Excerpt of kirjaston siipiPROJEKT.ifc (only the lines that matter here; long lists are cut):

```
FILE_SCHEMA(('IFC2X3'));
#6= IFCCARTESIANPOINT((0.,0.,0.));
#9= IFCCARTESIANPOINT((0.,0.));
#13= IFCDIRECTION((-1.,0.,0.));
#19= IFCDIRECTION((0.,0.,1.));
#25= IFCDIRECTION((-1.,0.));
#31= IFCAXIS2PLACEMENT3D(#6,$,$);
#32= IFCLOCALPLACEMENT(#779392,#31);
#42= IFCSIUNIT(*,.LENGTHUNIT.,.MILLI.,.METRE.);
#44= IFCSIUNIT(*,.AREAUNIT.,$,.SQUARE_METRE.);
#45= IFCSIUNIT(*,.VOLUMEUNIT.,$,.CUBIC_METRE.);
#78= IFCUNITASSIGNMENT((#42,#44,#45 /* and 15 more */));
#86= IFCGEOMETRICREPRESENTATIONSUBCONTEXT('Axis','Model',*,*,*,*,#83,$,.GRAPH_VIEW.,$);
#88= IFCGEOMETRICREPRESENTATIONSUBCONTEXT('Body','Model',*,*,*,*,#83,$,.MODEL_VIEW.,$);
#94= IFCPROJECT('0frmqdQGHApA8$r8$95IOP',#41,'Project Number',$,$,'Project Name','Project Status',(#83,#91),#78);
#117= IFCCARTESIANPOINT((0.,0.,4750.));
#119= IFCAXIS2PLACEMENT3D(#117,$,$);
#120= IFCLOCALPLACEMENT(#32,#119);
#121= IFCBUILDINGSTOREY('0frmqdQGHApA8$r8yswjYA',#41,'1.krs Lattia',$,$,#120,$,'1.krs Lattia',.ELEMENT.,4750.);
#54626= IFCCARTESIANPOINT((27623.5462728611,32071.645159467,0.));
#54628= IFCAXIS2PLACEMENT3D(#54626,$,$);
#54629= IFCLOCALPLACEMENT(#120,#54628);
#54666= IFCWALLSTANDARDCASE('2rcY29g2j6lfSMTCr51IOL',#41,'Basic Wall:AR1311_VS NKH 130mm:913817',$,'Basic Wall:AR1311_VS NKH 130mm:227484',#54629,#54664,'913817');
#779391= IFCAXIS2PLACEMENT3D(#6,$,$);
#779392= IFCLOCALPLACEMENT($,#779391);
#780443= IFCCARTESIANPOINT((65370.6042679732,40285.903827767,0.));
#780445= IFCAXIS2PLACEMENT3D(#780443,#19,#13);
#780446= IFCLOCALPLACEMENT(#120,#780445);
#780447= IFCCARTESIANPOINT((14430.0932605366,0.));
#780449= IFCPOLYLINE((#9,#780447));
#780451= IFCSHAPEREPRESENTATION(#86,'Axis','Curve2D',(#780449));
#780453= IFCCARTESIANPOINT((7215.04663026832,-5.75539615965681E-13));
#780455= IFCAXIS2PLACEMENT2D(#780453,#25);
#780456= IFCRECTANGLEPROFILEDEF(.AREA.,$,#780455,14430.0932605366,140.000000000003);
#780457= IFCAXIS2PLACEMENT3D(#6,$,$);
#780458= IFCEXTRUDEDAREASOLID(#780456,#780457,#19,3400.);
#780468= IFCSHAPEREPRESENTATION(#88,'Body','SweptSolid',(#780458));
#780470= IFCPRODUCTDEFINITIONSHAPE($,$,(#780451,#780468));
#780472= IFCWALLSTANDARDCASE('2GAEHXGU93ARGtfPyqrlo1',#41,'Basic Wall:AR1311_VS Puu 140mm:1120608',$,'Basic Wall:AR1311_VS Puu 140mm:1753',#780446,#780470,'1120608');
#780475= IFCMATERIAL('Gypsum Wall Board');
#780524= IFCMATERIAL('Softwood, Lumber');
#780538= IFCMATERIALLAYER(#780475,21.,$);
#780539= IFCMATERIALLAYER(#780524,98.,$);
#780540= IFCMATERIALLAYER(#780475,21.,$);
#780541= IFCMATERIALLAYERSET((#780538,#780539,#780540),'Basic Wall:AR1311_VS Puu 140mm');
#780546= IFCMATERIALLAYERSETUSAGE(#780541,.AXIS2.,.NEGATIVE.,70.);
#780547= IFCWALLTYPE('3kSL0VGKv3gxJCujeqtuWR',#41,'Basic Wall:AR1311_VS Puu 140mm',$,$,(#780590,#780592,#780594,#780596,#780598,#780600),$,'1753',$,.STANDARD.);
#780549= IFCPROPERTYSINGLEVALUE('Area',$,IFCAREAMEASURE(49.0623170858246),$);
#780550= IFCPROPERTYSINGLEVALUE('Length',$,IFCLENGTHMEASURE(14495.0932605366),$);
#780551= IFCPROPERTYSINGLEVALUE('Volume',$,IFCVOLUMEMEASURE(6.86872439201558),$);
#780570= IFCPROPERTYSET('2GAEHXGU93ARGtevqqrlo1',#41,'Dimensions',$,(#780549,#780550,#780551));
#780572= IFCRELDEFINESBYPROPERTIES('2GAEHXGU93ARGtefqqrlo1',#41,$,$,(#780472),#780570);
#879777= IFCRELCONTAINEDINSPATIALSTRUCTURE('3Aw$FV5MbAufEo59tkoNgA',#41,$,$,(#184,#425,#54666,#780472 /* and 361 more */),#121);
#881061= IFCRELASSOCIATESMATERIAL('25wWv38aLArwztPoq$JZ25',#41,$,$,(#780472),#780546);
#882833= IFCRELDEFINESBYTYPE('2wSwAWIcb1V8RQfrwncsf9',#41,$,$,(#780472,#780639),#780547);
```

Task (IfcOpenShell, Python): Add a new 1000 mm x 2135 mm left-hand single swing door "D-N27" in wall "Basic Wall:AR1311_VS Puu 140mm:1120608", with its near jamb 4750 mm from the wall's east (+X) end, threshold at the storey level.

```python
import numpy as np
import ifcopenshell
import ifcopenshell.api.feature
import ifcopenshell.api.geometry
import ifcopenshell.api.pset
import ifcopenshell.api.root
import ifcopenshell.api.spatial
import ifcopenshell.api.type
import ifcopenshell.geom
import ifcopenshell.util.element
import ifcopenshell.util.placement
import ifcopenshell.util.representation
import ifcopenshell.util.shape
import ifcopenshell.util.unit

model = ifcopenshell.open("kirjaston siipiPROJEKT.ifc")
unit_scale = ifcopenshell.util.unit.calculate_unit_scale(model)
area_scale = ifcopenshell.util.unit.calculate_unit_scale(model, "AREAUNIT")
volume_scale = ifcopenshell.util.unit.calculate_unit_scale(model, "VOLUMEUNIT")
settings = ifcopenshell.geom.settings()


def volume(element):
    """Net volume in cubic metres, openings subtracted."""
    shape = ifcopenshell.geom.create_shape(settings, element)
    return ifcopenshell.util.shape.get_volume(shape.geometry)


wall = model.by_guid("2GAEHXGU93ARGtfPyqrlo1")
storey = ifcopenshell.util.element.get_container(wall, ifc_class="IfcBuildingStorey")
context = ifcopenshell.util.representation.get_context(model, "Model", "Body", "MODEL_VIEW")
before = volume(wall)

width, height, from_end, sill = 1, 2.135, 4.75, 0.0  # metres

# The wall runs along its own X axis, and the end named is its -X end.
wall_shape = ifcopenshell.geom.create_shape(settings, wall)
x, y, z = ifcopenshell.util.shape.get_vertices(wall_shape.geometry).T
start = x.min() + from_end
face, thickness = float(y.min()), float(y.max() - y.min())
wall_matrix = ifcopenshell.util.placement.get_local_placement(wall.ObjectPlacement)
level = ifcopenshell.util.placement.get_local_placement(storey.ObjectPlacement)[2, 3]


def in_wall(x, y):
    """Placement at x, y metres in the wall's axes, at sill height."""
    matrix = wall_matrix.copy()
    matrix[:, 3] = wall_matrix @ np.array([x / unit_scale, y / unit_scale, 0.0, 1.0])
    matrix[2, 3] = level + sill / unit_scale
    return matrix


# Opening: a box that overshoots both wall faces by 50 mm.
opening = ifcopenshell.api.root.create_entity(model, ifc_class="IfcOpeningElement")
box = ifcopenshell.api.geometry.add_wall_representation(
    model, context=context, length=width, height=height, thickness=thickness + 0.1
)
ifcopenshell.api.geometry.assign_representation(model, product=opening, representation=box)
ifcopenshell.api.geometry.edit_object_placement(model, product=opening, matrix=in_wall(start, face - 0.05), is_si=False)
ifcopenshell.api.feature.add_feature(model, feature=opening, element=wall)

door = ifcopenshell.api.root.create_entity(model, ifc_class="IfcDoor", name="D-N27")
door.OverallWidth, door.OverallHeight = width / unit_scale, height / unit_scale
body = ifcopenshell.api.geometry.add_door_representation(
    model,
    context=context,
    overall_width=door.OverallWidth,
    overall_height=door.OverallHeight,
    operation_type="SINGLE_SWING_LEFT",
    lining_properties={"LiningDepth": thickness / unit_scale, "ThresholdDepth": thickness / unit_scale},
)
ifcopenshell.api.geometry.assign_representation(model, product=door, representation=body)
ifcopenshell.api.spatial.assign_container(model, products=[door], relating_structure=storey)
fills = ifcopenshell.api.feature.add_filling(model, opening=opening, element=door)
fills.OwnerHistory = door.OwnerHistory  # required in IFC2X3

# IFC2X3 keeps the operation on the door style.
style = ifcopenshell.api.root.create_entity(model, ifc_class="IfcDoorStyle", name="D-N27")
style.OperationType, style.ConstructionType = "SINGLE_SWING_LEFT", "NOTDEFINED"
style.ParameterTakesPrecedence = style.Sizeable = False
ifcopenshell.api.type.assign_type(model, related_objects=[door], relating_type=style)

# The lining spans the wall, so the door starts at the wall face.
ifcopenshell.api.geometry.edit_object_placement(model, product=door, matrix=in_wall(start, face), is_si=False)

after = volume(wall)

# Update the wall's stored quantities.
pset = model.by_id(ifcopenshell.util.element.get_pset(wall, "Dimensions", should_inherit=False)["id"])
ifcopenshell.api.pset.edit_pset(model, pset=pset, properties={
    "Area": model.create_entity("IfcAreaMeasure", after / thickness / area_scale),
    "Volume": model.create_entity("IfcVolumeMeasure", after / volume_scale),
})

print(f"wall volume {before:.3f} -> {after:.3f} m3")

model.write("kirjaston siipiPROJEKT_v2.ifc")
```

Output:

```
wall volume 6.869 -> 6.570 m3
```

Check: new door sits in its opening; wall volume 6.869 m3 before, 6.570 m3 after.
